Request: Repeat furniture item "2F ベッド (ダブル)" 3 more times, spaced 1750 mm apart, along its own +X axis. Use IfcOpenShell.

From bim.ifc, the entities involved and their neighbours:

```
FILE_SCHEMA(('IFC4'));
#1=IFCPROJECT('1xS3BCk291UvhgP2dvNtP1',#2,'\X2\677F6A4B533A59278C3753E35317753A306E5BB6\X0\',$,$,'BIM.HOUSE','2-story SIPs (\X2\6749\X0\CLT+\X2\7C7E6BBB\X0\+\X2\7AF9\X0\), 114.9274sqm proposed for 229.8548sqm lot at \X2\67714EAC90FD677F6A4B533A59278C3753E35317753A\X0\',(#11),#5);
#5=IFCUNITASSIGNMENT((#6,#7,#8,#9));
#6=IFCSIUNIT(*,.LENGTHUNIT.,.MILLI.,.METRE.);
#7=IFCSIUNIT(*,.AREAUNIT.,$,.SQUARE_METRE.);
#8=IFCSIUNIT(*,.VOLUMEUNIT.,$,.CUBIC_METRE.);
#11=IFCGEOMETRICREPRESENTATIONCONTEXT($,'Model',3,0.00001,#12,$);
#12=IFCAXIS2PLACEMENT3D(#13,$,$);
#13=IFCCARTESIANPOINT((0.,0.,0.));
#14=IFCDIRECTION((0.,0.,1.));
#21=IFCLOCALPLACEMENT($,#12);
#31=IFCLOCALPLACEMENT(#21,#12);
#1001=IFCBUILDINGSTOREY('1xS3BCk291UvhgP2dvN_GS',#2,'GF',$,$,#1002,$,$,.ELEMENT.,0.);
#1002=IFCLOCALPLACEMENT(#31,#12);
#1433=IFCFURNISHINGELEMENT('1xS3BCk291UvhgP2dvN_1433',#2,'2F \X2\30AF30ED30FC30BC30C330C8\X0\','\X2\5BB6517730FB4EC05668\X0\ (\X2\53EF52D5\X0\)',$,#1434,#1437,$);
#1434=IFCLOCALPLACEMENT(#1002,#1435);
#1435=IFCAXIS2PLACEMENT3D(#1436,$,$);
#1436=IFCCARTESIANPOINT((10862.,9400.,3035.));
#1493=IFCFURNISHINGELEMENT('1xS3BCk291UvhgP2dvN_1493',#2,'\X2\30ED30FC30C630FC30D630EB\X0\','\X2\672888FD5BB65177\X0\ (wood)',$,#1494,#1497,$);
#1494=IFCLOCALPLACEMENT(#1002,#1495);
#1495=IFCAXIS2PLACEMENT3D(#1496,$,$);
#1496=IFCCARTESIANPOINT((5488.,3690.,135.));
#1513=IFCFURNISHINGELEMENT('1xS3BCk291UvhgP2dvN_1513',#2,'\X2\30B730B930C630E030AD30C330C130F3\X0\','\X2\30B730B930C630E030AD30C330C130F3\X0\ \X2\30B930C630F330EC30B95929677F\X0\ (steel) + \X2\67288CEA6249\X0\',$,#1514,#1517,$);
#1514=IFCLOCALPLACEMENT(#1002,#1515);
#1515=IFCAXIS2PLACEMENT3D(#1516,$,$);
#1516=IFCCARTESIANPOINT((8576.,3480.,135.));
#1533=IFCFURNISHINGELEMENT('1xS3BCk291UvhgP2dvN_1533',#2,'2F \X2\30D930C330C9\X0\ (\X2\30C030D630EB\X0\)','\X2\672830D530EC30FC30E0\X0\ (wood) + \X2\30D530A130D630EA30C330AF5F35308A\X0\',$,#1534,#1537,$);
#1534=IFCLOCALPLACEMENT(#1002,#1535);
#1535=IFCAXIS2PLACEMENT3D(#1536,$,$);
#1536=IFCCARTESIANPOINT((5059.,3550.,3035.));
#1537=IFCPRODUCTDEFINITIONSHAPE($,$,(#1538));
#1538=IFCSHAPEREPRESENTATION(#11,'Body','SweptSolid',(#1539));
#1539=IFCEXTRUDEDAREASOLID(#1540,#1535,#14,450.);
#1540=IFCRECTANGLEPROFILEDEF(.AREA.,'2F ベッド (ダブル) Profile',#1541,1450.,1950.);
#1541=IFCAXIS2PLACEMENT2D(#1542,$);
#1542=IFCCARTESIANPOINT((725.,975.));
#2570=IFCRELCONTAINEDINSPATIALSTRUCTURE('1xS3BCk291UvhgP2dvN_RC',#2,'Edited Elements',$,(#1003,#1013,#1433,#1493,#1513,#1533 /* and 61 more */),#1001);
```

```python
import ifcopenshell
import ifcopenshell.api.geometry
import ifcopenshell.api.root
import ifcopenshell.util.element
import ifcopenshell.util.placement

model = ifcopenshell.open("bim.ifc")


def reuse_history(source, copy):
    """copy_class also copies each property set's owner history, people and application; keep the originals."""
    for rel in copy.IsDefinedBy:
        if rel.is_a("IfcRelDefinesByProperties") and (history := rel.RelatingPropertyDefinition.OwnerHistory):
            rel.RelatingPropertyDefinition.OwnerHistory = source.OwnerHistory
            ifcopenshell.util.element.remove_deep2(model, history)


source = model.by_guid("1xS3BCk291UvhgP2dvN_1533")
base = ifcopenshell.util.placement.get_local_placement(source.ObjectPlacement)
step = base[:3, 0] * 1750.0

for i in range(1, 4):
    copy = ifcopenshell.api.root.copy_class(model, product=source)
    copy.Representation = ifcopenshell.util.element.copy_deep(
        model, source.Representation, exclude=["IfcGeometricRepresentationContext", "IfcRepresentationMap"]
    )
    reuse_history(source, copy)
    matrix = base.copy()
    matrix[:3, 3] += i * step
    print("added at", matrix[:3, 3].round(3) + 0.0)
    ifcopenshell.api.geometry.edit_object_placement(model, product=copy, matrix=matrix, is_si=False)

model.write("bim_edited.ifc")
```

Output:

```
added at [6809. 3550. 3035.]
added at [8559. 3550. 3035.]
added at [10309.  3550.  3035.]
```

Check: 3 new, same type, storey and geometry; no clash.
